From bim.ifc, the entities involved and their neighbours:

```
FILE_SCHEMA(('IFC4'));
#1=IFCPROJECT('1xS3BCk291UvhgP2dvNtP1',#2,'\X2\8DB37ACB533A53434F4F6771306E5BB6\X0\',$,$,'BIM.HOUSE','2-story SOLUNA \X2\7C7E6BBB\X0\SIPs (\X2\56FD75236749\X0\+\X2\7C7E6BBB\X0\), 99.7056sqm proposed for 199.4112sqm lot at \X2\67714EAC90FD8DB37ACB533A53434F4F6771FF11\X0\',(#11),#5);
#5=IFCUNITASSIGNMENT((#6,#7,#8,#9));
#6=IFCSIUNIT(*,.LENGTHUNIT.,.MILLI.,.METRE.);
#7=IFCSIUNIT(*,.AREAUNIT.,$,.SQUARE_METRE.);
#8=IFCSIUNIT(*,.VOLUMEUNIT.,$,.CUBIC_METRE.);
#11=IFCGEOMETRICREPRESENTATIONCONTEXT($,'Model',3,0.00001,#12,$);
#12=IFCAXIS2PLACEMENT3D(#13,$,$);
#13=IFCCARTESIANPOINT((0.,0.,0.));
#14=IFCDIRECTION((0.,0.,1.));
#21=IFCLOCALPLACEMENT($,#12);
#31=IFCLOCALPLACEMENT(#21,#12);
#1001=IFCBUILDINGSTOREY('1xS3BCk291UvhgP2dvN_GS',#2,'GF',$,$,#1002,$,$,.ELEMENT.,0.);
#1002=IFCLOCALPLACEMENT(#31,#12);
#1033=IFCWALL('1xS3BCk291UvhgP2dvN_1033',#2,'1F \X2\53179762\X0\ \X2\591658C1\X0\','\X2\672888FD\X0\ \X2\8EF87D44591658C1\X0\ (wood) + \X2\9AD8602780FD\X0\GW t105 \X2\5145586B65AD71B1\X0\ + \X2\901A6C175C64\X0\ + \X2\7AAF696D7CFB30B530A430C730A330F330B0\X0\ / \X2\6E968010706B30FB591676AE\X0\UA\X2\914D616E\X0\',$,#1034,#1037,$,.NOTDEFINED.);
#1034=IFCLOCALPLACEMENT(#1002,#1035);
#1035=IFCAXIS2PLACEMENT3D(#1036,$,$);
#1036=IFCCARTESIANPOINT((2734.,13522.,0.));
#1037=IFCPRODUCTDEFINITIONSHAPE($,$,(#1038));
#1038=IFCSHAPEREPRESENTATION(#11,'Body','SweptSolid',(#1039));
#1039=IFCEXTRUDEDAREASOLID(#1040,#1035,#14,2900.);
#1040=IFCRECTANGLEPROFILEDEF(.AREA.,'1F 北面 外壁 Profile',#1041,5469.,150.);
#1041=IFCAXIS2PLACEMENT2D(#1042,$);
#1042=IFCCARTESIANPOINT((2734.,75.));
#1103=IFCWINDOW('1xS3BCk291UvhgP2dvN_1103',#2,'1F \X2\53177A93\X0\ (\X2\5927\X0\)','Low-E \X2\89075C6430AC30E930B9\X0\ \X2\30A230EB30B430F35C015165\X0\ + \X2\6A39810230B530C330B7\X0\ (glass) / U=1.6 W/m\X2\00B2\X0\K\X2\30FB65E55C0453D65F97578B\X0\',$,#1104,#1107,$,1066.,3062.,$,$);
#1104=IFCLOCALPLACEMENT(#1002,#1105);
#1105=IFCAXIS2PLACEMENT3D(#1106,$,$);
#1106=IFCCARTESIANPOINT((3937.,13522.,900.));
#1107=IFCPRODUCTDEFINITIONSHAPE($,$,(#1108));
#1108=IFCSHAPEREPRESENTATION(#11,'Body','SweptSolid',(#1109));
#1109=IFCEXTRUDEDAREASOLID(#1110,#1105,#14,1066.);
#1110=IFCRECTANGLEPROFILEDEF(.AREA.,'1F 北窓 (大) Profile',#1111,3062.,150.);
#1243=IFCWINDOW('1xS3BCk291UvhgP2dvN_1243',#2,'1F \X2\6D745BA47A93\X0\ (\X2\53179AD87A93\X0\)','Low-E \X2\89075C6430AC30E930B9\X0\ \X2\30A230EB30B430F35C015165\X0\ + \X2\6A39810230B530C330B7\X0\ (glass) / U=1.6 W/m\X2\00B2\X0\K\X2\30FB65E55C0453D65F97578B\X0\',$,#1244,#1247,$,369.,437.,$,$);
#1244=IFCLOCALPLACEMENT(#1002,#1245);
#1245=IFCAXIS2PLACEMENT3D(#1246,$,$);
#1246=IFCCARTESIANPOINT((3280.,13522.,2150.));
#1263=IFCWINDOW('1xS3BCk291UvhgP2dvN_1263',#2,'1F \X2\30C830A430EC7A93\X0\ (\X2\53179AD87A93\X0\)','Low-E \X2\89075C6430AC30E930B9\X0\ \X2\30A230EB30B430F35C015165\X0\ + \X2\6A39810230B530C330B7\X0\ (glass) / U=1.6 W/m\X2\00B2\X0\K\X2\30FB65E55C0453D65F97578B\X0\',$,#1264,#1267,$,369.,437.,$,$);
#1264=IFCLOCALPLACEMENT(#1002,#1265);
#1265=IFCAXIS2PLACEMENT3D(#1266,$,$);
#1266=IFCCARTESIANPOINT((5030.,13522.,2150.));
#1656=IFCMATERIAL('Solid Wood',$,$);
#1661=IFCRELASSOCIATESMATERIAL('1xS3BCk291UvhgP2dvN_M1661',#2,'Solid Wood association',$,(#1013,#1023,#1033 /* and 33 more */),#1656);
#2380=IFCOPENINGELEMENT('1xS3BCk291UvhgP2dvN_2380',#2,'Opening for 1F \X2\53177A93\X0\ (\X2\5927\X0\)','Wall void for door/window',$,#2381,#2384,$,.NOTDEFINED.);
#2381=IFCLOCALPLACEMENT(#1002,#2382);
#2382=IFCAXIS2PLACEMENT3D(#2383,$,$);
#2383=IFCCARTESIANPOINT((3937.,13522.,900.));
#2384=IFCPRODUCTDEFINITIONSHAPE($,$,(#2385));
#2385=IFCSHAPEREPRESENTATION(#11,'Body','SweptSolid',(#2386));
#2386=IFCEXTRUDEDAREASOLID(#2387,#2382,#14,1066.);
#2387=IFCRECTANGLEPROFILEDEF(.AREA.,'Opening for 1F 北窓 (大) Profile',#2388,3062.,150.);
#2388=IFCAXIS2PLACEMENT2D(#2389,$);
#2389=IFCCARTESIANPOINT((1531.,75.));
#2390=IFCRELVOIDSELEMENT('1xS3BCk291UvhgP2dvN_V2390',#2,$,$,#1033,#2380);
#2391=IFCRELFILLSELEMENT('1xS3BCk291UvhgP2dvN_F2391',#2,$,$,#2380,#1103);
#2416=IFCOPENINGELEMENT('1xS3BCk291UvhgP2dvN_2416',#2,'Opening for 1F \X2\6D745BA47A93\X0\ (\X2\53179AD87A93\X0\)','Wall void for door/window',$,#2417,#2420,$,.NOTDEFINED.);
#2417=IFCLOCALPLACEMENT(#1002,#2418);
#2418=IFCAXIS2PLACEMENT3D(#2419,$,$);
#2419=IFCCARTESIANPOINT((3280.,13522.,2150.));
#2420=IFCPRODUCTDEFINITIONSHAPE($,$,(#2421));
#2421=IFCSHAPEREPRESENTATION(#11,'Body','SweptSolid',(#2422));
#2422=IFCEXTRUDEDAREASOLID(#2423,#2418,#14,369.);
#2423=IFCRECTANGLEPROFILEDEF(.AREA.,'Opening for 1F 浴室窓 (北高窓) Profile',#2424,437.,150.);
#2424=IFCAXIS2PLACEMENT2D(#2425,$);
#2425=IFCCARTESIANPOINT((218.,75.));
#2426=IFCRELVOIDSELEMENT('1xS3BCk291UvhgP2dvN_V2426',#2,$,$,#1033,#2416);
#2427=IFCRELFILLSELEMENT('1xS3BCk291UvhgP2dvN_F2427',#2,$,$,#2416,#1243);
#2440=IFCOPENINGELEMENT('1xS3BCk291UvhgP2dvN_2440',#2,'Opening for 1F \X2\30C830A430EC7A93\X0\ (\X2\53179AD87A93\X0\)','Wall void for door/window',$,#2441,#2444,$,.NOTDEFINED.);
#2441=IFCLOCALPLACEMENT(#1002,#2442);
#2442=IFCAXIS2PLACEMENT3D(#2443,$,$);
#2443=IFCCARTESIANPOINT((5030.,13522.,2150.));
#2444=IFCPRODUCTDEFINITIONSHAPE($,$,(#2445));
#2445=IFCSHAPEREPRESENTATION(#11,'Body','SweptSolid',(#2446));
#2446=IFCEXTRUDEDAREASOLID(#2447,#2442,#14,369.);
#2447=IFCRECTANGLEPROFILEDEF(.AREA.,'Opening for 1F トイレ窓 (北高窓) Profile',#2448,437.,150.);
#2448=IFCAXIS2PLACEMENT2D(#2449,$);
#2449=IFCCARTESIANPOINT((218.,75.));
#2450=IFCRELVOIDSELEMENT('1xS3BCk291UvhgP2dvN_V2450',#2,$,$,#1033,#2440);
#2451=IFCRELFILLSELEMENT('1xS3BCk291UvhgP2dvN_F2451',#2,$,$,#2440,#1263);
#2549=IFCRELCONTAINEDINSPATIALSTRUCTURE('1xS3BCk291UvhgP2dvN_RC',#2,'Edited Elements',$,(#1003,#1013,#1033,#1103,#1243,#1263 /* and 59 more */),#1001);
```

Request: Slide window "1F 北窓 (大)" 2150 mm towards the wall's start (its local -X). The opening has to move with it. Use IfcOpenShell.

```python
import ifcopenshell
import ifcopenshell.api.geometry
import ifcopenshell.util.placement
import ifcopenshell.util.unit

model = ifcopenshell.open("bim.ifc")
unit_scale = ifcopenshell.util.unit.calculate_unit_scale(model)

window = model.by_guid("1xS3BCk291UvhgP2dvN_1103")
opening = window.FillsVoids[0].RelatingOpeningElement
wall = opening.VoidsElements[0].RelatingBuildingElement

wall_matrix = ifcopenshell.util.placement.get_local_placement(wall.ObjectPlacement)
shift = wall_matrix[:3, 0] * -2.15 / unit_scale
before = ifcopenshell.util.placement.get_local_placement(window.ObjectPlacement)[:3, 3].copy()

# The window is not placed relative to its opening, so move both.
for product in (opening, window):
    matrix = ifcopenshell.util.placement.get_local_placement(product.ObjectPlacement)
    matrix[:3, 3] += shift
    ifcopenshell.api.geometry.edit_object_placement(model, product=product, matrix=matrix, is_si=False)

after = ifcopenshell.util.placement.get_local_placement(window.ObjectPlacement)[:3, 3]
print("window moved by", (after - before).round(3) + 0.0)

model.write("bim_edited.ifc")
```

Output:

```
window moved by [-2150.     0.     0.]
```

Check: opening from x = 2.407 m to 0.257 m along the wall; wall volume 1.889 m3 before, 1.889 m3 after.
